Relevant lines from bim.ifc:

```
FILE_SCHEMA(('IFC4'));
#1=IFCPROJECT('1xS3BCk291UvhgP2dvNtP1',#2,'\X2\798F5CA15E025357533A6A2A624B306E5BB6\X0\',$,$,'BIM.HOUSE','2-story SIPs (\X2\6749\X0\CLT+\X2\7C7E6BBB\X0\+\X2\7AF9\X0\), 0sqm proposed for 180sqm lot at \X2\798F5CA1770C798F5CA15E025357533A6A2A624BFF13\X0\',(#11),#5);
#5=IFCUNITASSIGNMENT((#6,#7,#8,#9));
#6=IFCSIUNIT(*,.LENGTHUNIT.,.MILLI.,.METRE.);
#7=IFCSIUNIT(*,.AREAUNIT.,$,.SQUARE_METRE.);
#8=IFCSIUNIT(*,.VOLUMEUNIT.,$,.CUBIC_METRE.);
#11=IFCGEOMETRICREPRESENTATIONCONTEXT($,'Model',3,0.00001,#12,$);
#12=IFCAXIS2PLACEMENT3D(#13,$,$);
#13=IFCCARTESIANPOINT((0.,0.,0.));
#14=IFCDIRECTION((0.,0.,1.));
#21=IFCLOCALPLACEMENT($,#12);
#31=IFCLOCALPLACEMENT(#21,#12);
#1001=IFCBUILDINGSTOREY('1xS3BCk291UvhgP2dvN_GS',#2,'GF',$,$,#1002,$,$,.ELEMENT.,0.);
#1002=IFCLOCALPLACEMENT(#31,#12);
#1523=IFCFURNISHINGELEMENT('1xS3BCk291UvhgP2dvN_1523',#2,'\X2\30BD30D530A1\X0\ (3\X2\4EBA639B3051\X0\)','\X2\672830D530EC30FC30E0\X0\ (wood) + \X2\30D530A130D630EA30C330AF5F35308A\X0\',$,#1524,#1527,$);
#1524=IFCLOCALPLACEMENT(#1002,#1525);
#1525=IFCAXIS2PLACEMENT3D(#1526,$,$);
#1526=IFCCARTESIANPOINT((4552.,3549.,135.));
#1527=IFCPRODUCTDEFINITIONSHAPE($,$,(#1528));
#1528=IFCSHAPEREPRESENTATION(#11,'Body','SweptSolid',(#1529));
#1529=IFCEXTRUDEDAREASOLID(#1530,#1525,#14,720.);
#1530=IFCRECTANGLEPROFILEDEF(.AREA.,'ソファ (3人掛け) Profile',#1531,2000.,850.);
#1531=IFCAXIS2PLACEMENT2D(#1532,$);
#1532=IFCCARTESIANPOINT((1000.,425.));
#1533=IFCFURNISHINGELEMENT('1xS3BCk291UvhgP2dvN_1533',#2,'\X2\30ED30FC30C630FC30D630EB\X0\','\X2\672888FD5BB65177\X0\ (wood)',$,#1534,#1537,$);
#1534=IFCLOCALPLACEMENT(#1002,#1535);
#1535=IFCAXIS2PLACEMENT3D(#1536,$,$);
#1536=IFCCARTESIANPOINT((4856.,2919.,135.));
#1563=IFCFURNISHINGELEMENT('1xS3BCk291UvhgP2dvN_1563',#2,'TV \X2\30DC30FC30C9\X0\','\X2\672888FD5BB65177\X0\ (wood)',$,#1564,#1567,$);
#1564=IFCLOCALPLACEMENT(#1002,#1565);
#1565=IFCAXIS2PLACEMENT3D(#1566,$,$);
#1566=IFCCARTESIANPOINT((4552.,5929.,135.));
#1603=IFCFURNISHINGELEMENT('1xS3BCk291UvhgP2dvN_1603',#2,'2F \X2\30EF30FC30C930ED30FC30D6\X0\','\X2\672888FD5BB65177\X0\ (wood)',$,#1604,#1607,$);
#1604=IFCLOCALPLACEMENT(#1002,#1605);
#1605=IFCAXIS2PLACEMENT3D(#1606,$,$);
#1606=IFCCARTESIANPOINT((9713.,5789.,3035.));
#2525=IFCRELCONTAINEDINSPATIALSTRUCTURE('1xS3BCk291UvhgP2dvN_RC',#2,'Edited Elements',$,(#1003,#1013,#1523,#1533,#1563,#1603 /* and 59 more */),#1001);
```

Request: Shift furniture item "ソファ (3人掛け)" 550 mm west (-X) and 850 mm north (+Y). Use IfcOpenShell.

```python
import ifcopenshell
import ifcopenshell.api.geometry
import ifcopenshell.util.placement

model = ifcopenshell.open("bim.ifc")

item = model.by_guid("1xS3BCk291UvhgP2dvN_1523")
matrix = ifcopenshell.util.placement.get_local_placement(item.ObjectPlacement)
matrix[0, 3] -= 550.0
matrix[1, 3] += 850.0
ifcopenshell.api.geometry.edit_object_placement(model, product=item, matrix=matrix, is_si=False)

print(ifcopenshell.util.placement.get_local_placement(item.ObjectPlacement).round(3) + 0.0)

model.write("bim_v2.ifc")
```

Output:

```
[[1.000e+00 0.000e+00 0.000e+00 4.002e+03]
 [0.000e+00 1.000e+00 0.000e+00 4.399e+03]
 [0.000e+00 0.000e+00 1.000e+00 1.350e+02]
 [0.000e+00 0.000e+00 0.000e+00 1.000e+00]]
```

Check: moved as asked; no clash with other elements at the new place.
